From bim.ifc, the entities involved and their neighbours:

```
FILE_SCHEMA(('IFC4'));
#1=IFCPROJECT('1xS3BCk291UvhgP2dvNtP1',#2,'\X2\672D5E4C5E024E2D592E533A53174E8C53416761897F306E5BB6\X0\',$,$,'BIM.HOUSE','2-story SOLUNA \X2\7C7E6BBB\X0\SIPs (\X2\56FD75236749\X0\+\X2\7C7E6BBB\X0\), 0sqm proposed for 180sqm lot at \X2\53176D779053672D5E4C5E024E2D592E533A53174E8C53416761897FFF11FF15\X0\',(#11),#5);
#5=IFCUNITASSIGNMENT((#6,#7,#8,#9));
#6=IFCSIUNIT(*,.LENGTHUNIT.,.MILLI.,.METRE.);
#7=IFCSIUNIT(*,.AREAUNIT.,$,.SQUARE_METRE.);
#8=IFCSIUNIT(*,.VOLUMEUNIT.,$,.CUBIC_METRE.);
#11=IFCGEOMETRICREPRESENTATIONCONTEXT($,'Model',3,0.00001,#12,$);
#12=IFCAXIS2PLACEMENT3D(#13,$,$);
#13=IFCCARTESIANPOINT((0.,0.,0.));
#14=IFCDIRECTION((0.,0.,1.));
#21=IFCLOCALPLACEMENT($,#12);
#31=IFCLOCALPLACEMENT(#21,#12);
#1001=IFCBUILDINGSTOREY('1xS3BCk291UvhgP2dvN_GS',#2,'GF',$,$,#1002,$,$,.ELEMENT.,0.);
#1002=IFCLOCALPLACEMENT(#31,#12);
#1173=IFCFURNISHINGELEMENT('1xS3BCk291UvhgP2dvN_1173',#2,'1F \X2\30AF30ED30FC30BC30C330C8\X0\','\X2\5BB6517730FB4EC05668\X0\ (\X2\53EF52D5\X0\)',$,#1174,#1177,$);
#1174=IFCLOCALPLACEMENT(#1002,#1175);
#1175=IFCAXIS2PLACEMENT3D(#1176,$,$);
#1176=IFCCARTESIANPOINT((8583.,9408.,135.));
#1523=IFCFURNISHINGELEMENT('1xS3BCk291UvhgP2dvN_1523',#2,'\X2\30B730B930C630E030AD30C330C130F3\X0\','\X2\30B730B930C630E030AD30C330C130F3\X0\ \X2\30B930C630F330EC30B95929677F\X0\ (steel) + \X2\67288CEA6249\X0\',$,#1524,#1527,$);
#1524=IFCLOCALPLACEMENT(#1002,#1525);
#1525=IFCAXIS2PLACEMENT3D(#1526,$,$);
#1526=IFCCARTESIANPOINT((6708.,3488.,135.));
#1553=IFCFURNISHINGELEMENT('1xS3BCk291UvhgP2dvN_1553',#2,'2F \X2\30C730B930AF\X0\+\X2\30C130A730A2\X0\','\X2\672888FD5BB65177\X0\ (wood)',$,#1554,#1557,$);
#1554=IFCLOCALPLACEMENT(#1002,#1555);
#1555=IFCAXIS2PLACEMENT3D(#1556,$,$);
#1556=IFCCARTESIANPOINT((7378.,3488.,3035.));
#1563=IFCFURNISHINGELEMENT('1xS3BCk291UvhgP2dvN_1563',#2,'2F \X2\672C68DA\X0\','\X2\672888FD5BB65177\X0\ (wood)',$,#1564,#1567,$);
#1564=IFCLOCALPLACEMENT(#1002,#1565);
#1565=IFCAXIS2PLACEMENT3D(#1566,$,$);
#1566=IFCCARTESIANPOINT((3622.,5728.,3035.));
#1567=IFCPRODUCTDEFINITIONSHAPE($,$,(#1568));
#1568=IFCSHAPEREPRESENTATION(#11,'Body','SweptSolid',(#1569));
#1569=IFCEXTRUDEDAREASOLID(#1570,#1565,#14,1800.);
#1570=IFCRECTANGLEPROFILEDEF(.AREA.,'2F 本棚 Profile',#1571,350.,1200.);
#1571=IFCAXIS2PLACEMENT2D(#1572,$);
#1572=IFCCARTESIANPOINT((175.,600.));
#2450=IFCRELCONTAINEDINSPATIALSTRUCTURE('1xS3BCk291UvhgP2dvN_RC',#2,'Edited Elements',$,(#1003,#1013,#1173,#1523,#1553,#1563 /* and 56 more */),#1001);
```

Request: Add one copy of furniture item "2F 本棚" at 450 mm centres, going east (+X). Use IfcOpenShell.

```python
import numpy as np
import ifcopenshell
import ifcopenshell.api.geometry
import ifcopenshell.api.root
import ifcopenshell.util.element
import ifcopenshell.util.placement

model = ifcopenshell.open("bim.ifc")


def reuse_history(source, copy):
    """copy_class also copies each property set's owner history, people and application; keep the originals."""
    for rel in copy.IsDefinedBy:
        if rel.is_a("IfcRelDefinesByProperties") and (history := rel.RelatingPropertyDefinition.OwnerHistory):
            rel.RelatingPropertyDefinition.OwnerHistory = source.OwnerHistory
            ifcopenshell.util.element.remove_deep2(model, history)


source = model.by_id(1563)
base = ifcopenshell.util.placement.get_local_placement(source.ObjectPlacement)
step = np.array([1.0, 0.0, 0.0]) * 450.0

for i in range(1, 2):
    copy = ifcopenshell.api.root.copy_class(model, product=source)
    copy.Representation = ifcopenshell.util.element.copy_deep(
        model, source.Representation, exclude=["IfcGeometricRepresentationContext", "IfcRepresentationMap"]
    )
    reuse_history(source, copy)
    matrix = base.copy()
    matrix[:3, 3] += i * step
    print("added at", matrix[:3, 3].round(3) + 0.0)
    ifcopenshell.api.geometry.edit_object_placement(model, product=copy, matrix=matrix, is_si=False)

model.write("bim_rev.ifc")
```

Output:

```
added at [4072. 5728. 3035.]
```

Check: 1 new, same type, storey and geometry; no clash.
